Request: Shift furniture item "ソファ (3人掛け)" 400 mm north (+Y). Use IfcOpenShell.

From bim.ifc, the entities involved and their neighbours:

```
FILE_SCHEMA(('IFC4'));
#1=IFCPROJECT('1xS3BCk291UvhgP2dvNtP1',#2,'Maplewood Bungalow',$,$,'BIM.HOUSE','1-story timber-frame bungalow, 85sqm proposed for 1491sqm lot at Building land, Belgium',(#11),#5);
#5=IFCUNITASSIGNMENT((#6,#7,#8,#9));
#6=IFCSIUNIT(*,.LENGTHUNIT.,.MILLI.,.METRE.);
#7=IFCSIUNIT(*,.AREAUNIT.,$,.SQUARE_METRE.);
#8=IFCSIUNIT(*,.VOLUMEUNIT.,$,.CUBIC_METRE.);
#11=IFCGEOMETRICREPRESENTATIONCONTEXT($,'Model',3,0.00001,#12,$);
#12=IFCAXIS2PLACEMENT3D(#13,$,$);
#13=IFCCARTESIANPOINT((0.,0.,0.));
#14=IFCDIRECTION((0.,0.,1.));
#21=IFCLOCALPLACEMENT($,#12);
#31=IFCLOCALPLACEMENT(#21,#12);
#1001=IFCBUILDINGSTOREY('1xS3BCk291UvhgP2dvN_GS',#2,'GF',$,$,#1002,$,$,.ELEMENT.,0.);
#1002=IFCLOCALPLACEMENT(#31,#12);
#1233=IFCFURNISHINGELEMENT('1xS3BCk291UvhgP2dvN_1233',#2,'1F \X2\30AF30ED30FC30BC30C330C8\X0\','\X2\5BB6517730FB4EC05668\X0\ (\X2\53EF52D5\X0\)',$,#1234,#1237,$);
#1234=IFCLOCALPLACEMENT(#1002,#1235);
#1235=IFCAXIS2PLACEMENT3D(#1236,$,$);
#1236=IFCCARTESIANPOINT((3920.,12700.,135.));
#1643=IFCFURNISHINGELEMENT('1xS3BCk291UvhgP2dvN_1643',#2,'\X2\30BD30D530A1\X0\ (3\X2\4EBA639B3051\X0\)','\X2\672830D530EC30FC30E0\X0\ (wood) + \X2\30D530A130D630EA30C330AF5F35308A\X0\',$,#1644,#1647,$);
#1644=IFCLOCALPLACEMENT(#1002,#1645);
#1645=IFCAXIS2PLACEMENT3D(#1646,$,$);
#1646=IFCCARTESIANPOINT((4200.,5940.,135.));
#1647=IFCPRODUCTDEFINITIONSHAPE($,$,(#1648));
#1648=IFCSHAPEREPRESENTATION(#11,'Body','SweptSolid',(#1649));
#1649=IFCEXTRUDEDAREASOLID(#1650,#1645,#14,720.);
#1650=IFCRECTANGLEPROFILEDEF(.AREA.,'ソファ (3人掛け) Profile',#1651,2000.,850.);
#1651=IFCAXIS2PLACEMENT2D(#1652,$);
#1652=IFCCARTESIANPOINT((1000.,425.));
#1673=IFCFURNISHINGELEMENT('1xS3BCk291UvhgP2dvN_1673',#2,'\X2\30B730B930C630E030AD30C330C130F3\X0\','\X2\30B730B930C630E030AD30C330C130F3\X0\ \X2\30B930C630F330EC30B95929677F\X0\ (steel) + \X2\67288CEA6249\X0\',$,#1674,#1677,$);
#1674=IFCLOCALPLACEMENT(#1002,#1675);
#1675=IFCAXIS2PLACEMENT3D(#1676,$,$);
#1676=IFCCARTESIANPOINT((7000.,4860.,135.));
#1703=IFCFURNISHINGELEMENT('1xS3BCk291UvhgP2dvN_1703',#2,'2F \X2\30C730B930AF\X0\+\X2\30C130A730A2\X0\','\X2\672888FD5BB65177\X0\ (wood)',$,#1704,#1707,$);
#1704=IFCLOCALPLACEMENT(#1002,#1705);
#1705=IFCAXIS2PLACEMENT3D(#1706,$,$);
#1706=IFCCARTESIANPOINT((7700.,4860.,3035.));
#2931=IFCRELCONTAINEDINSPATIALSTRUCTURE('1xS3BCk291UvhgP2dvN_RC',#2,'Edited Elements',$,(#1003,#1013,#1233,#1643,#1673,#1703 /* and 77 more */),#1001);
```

```python
import ifcopenshell
import ifcopenshell.api.geometry
import ifcopenshell.util.placement
import ifcopenshell.util.unit

model = ifcopenshell.open("bim.ifc")
unit_scale = ifcopenshell.util.unit.calculate_unit_scale(model)

item = model.by_guid("1xS3BCk291UvhgP2dvN_1643")
matrix = ifcopenshell.util.placement.get_local_placement(item.ObjectPlacement)
matrix[1, 3] += 0.4 / unit_scale
ifcopenshell.api.geometry.edit_object_placement(model, product=item, matrix=matrix, is_si=False)

print(ifcopenshell.util.placement.get_local_placement(item.ObjectPlacement).round(3) + 0.0)

model.write("bim_rev.ifc")
```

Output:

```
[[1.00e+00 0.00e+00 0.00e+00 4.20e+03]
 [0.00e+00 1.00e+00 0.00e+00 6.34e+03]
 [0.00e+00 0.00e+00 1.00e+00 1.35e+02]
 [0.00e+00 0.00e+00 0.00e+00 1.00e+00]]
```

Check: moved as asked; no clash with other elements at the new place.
